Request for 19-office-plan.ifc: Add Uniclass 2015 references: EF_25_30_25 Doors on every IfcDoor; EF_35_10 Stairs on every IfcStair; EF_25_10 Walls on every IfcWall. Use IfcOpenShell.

First a look at what the model holds.

```python
import ifcopenshell

model = ifcopenshell.open("19-office-plan.ifc")
print(model.schema)
print("classifications:", [c.Name for c in model.by_type("IfcClassification")])
for ifc_class in ("IfcDoor", "IfcRoof", "IfcStair", "IfcWall", "IfcWindow"):
    print(ifc_class, len(model.by_type(ifc_class)))
```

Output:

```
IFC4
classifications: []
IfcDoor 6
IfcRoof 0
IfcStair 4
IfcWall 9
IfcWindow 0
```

```python
import ifcopenshell
import ifcopenshell.api.classification

model = ifcopenshell.open("19-office-plan.ifc")

system = ifcopenshell.api.classification.add_classification(model, classification="Uniclass 2015")

codes = {
    "IfcDoor": ("EF_25_30_25", "Doors"),
    "IfcStair": ("EF_35_10", "Stairs"),
    "IfcWall": ("EF_25_10", "Walls"),
}
for ifc_class, (code, name) in codes.items():
    products = model.by_type(ifc_class)
    ifcopenshell.api.classification.add_reference(
        model, products=products, classification=system, identification=code, name=name
    )
    print(code, len(products))

model.write("19-office-plan_v2.ifc")
```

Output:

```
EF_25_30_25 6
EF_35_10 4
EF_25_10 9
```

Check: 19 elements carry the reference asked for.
